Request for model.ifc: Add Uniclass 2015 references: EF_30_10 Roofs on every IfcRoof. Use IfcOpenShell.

First a look at what the model holds.

```python
import ifcopenshell

model = ifcopenshell.open("model.ifc")
print(model.schema)
print("classifications:", [c.Name for c in model.by_type("IfcClassification")])
for ifc_class in ("IfcDoor", "IfcRoof", "IfcStair", "IfcWall", "IfcWindow"):
    print(ifc_class, len(model.by_type(ifc_class)))
```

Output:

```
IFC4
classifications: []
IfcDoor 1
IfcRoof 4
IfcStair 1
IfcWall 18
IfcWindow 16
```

```python
import ifcopenshell
import ifcopenshell.api.classification

model = ifcopenshell.open("model.ifc")

system = ifcopenshell.api.classification.add_classification(model, classification="Uniclass 2015")

codes = {
    "IfcRoof": ("EF_30_10", "Roofs"),
}
for ifc_class, (code, name) in codes.items():
    products = model.by_type(ifc_class)
    ifcopenshell.api.classification.add_reference(
        model, products=products, classification=system, identification=code, name=name
    )
    print(code, len(products))

model.write("model_v2.ifc")
```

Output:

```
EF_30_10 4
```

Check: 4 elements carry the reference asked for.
